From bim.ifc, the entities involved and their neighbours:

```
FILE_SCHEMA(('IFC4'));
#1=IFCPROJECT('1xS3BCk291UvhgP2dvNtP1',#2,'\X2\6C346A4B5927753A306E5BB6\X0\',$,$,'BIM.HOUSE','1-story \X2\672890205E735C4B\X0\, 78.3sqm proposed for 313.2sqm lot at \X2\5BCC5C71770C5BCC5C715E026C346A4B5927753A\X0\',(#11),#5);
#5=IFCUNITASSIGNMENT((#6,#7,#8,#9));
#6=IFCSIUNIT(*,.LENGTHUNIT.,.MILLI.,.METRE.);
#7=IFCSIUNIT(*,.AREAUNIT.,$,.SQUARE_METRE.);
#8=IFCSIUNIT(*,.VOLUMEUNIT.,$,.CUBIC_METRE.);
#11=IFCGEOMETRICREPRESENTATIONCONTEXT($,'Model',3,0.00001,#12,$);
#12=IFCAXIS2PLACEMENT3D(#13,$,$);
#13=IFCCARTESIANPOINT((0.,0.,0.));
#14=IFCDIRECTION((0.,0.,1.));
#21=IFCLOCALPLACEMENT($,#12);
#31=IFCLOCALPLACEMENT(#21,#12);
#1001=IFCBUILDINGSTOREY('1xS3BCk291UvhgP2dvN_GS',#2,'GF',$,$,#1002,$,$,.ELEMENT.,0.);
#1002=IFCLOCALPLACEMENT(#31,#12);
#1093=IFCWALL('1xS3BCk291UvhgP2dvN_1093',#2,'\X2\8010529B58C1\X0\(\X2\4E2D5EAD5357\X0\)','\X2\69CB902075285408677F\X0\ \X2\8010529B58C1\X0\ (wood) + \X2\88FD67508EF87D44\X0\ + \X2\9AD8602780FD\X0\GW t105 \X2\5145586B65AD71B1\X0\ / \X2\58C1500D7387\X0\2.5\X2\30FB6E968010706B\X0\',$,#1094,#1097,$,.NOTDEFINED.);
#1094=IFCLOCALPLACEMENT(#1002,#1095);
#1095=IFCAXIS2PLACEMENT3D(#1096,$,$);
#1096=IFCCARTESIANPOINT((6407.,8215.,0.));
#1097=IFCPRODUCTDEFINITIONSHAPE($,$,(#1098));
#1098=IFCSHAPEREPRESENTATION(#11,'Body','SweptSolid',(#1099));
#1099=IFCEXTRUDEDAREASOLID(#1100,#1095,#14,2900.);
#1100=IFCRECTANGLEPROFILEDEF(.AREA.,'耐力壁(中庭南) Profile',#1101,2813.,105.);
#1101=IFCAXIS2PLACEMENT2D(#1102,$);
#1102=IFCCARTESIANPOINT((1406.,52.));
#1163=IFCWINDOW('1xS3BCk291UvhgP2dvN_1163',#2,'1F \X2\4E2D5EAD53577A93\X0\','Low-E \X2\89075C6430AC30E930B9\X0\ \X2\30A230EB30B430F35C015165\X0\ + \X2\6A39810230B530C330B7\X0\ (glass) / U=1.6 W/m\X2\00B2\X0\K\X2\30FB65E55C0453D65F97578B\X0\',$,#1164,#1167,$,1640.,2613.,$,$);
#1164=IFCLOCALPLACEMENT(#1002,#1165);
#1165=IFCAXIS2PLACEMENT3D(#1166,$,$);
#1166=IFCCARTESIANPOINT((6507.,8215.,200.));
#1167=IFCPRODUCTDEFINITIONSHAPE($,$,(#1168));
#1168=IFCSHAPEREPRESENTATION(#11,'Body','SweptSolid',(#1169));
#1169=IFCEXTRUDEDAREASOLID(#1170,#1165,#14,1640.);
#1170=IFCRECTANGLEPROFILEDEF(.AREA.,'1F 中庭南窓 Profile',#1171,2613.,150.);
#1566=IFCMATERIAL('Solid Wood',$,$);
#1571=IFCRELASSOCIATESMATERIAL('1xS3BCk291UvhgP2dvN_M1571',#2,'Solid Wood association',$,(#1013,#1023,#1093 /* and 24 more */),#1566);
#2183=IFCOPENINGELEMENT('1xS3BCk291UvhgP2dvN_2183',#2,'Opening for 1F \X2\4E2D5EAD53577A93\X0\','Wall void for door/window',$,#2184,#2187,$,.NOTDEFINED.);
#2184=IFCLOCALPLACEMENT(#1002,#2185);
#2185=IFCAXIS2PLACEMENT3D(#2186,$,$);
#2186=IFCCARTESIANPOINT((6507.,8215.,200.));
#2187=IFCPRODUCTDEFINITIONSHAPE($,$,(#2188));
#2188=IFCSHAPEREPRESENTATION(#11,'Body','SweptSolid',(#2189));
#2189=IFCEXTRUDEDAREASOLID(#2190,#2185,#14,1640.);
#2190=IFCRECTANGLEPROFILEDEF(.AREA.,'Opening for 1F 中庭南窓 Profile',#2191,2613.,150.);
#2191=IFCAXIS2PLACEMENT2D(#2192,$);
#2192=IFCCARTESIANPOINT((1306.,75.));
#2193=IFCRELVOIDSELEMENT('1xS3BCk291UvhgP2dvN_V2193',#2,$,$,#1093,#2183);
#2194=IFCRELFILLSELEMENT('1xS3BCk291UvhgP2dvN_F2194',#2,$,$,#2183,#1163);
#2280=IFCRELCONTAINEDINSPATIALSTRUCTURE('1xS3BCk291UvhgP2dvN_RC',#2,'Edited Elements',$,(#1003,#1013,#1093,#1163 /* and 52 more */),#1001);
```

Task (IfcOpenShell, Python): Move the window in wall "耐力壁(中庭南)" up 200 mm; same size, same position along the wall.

```python
import numpy as np
import ifcopenshell
import ifcopenshell.api.geometry
import ifcopenshell.util.placement
import ifcopenshell.util.unit

model = ifcopenshell.open("bim.ifc")
unit_scale = ifcopenshell.util.unit.calculate_unit_scale(model)

window = model.by_guid("1xS3BCk291UvhgP2dvN_1163")
opening = window.FillsVoids[0].RelatingOpeningElement
dz = 200.0

shift = np.array([0.0, 0.0, dz])
# The window is not placed relative to its opening, so move both.
for product in (opening, window):
    matrix = ifcopenshell.util.placement.get_local_placement(product.ObjectPlacement)
    matrix[:3, 3] += shift
    ifcopenshell.api.geometry.edit_object_placement(model, product=product, matrix=matrix, is_si=False)

print(f"moved by {dz * unit_scale:+.3f} m")

model.write("bim-out.ifc")
```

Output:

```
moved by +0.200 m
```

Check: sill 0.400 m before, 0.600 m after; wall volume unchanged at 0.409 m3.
